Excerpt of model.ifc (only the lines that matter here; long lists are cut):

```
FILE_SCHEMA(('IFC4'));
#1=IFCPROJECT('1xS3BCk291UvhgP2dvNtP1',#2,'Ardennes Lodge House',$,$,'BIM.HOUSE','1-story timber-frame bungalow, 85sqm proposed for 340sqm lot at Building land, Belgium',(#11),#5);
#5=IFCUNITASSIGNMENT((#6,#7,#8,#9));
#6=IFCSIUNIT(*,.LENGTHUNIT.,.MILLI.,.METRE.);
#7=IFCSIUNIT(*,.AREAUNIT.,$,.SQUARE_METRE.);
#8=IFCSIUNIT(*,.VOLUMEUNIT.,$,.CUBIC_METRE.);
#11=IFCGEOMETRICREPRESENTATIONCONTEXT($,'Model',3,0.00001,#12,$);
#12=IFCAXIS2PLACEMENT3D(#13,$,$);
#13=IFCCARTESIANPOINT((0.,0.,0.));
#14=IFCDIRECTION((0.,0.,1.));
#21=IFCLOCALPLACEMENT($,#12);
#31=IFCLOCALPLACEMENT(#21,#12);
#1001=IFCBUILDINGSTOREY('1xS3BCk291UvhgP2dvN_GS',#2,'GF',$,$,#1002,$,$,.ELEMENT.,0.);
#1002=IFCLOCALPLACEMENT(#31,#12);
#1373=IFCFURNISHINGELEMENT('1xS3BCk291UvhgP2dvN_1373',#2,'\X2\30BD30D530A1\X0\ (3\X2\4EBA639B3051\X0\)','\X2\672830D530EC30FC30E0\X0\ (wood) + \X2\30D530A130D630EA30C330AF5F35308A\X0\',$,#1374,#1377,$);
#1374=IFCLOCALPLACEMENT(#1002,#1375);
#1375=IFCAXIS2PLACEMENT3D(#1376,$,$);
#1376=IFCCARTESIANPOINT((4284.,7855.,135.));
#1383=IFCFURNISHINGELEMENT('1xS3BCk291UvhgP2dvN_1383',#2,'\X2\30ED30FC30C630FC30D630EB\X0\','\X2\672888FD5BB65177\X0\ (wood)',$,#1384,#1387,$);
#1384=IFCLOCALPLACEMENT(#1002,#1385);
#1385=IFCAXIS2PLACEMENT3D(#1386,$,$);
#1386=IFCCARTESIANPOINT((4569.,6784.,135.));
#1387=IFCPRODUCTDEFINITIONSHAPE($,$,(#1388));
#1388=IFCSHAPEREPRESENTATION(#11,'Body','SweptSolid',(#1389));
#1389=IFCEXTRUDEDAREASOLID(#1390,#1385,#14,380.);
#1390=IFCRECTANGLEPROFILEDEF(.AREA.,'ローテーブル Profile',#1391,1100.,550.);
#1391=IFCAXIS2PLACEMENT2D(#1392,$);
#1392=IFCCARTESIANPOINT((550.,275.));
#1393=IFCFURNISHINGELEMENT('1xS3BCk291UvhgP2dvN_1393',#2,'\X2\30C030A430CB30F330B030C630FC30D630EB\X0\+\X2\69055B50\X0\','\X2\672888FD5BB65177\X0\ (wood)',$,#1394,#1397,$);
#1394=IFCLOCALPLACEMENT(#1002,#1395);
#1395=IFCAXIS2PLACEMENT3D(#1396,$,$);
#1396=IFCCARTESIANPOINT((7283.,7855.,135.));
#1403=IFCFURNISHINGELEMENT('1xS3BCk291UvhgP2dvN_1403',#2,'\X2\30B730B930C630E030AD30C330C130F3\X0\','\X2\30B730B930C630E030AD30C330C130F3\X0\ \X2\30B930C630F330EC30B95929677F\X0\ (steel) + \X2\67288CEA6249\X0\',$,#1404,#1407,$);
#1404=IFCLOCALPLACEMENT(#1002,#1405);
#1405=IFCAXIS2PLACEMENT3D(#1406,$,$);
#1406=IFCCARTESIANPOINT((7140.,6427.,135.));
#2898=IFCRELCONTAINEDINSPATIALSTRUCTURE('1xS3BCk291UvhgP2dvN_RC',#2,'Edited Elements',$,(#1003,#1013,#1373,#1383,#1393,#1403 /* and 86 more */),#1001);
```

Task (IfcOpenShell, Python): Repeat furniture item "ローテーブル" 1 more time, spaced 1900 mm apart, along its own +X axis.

```python
import ifcopenshell
import ifcopenshell.api.geometry
import ifcopenshell.api.root
import ifcopenshell.util.element
import ifcopenshell.util.placement
import ifcopenshell.util.unit

model = ifcopenshell.open("model.ifc")
unit_scale = ifcopenshell.util.unit.calculate_unit_scale(model)


def reuse_history(source, copy):
    """copy_class also copies each property set's owner history, people and application; keep the originals."""
    for rel in copy.IsDefinedBy:
        if rel.is_a("IfcRelDefinesByProperties") and (history := rel.RelatingPropertyDefinition.OwnerHistory):
            rel.RelatingPropertyDefinition.OwnerHistory = source.OwnerHistory
            ifcopenshell.util.element.remove_deep2(model, history)


source = model.by_guid("1xS3BCk291UvhgP2dvN_1383")
base = ifcopenshell.util.placement.get_local_placement(source.ObjectPlacement)
step = base[:3, 0] * 1.9 / unit_scale

for i in range(1, 2):
    copy = ifcopenshell.api.root.copy_class(model, product=source)
    copy.Representation = ifcopenshell.util.element.copy_deep(
        model, source.Representation, exclude=["IfcGeometricRepresentationContext", "IfcRepresentationMap"]
    )
    reuse_history(source, copy)
    matrix = base.copy()
    matrix[:3, 3] += i * step
    print("added at", matrix[:3, 3].round(3) + 0.0)
    ifcopenshell.api.geometry.edit_object_placement(model, product=copy, matrix=matrix, is_si=False)

model.write("model_v2.ifc")
```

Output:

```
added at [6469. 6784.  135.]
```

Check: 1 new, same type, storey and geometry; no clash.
